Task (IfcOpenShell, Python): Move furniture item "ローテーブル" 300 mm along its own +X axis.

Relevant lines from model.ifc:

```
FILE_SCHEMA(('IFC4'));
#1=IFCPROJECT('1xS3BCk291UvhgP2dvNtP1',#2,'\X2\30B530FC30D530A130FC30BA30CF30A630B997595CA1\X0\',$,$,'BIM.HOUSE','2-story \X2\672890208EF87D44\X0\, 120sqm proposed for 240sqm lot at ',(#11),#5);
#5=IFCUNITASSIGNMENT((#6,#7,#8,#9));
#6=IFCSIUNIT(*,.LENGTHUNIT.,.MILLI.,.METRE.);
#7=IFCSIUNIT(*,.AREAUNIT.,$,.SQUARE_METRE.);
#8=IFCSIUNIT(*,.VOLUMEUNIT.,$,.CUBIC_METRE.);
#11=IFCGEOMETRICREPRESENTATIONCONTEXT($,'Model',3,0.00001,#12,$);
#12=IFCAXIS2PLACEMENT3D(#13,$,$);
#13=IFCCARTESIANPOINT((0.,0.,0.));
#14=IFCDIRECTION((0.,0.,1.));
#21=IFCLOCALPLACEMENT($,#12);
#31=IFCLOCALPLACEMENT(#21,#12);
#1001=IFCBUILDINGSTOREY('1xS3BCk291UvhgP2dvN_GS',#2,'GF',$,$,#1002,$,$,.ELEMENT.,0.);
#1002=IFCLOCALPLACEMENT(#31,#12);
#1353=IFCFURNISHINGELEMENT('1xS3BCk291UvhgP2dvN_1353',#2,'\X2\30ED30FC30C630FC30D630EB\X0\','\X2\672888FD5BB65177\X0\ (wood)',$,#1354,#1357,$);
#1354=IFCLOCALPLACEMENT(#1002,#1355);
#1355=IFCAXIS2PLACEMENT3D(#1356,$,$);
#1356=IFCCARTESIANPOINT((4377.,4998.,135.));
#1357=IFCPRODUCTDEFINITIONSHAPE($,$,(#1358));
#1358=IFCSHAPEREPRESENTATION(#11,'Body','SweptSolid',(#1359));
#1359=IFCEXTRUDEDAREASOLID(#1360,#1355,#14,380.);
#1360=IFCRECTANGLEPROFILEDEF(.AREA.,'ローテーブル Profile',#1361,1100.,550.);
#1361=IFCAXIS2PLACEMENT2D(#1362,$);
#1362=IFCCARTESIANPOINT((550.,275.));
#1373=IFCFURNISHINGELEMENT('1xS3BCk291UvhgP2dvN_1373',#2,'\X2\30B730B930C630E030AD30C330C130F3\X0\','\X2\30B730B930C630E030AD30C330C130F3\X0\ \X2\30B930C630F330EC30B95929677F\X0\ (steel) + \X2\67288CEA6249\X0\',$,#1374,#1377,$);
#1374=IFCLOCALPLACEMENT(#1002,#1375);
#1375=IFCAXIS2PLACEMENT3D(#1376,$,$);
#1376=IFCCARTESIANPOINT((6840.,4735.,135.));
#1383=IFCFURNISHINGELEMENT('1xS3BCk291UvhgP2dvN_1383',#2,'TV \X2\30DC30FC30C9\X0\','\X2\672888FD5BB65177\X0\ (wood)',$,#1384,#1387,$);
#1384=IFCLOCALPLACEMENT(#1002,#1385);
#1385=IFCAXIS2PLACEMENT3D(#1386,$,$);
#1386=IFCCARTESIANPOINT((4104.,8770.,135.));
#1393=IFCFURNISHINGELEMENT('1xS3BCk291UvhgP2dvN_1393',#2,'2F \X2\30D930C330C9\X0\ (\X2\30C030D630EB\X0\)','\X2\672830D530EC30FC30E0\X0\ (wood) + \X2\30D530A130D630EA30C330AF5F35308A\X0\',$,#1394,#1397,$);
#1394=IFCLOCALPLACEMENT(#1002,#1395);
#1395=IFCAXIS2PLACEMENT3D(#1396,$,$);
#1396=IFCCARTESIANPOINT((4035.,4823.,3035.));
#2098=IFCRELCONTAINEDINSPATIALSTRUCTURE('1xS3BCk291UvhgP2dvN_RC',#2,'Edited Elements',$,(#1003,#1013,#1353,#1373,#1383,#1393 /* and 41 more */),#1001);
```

```python
import ifcopenshell
import ifcopenshell.api.geometry
import ifcopenshell.util.placement

model = ifcopenshell.open("model.ifc")

item = model.by_guid("1xS3BCk291UvhgP2dvN_1353")
matrix = ifcopenshell.util.placement.get_local_placement(item.ObjectPlacement)
matrix[:3, 3] += matrix[:3, 0] * 300.0
ifcopenshell.api.geometry.edit_object_placement(model, product=item, matrix=matrix, is_si=False)

print(ifcopenshell.util.placement.get_local_placement(item.ObjectPlacement).round(3) + 0.0)

model.write("model_rev.ifc")
```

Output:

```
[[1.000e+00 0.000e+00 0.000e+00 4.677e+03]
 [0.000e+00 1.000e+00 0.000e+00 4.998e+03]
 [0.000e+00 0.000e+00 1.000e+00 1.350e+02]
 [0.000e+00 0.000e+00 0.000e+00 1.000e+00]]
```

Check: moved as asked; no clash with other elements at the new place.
